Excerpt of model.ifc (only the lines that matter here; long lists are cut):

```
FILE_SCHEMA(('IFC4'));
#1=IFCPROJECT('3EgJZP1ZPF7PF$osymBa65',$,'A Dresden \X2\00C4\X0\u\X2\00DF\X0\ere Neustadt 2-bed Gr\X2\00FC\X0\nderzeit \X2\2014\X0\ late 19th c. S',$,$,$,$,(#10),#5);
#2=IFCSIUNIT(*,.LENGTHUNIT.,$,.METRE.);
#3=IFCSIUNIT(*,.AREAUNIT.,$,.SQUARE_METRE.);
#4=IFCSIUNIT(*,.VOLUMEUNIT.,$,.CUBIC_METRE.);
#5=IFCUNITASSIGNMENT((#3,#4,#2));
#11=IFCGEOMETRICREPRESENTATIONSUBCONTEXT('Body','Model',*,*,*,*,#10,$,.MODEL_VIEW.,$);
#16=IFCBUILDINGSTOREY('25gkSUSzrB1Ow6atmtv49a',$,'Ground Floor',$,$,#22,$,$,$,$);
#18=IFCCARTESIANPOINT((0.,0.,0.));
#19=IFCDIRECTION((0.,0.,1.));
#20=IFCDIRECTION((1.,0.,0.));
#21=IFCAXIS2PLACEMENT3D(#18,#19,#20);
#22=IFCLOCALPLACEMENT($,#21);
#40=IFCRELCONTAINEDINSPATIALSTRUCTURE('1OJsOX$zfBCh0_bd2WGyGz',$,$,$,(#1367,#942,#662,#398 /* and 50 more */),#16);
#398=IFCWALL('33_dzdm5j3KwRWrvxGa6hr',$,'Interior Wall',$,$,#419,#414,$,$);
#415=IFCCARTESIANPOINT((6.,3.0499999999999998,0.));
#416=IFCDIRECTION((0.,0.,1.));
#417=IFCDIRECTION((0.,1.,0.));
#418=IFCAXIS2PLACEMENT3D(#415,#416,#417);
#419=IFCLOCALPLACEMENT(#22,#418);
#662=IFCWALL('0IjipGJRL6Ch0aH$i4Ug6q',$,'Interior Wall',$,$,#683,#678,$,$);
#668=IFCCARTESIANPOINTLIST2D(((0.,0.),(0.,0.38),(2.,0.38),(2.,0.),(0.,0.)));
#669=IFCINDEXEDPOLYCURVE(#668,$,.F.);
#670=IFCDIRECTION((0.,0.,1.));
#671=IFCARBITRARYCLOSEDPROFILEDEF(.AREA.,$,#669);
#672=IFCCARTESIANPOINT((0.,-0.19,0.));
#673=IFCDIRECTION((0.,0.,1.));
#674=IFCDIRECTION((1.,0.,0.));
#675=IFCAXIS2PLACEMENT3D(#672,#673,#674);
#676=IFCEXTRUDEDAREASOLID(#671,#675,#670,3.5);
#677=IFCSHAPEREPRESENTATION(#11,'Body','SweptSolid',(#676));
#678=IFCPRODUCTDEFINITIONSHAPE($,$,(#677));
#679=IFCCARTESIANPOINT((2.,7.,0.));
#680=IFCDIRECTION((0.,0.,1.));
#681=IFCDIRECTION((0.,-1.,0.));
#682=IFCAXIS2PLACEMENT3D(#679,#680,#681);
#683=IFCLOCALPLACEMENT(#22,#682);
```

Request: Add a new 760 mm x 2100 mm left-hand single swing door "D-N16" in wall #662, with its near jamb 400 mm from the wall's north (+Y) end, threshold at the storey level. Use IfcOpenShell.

```python
import numpy as np
import ifcopenshell
import ifcopenshell.api.feature
import ifcopenshell.api.geometry
import ifcopenshell.api.root
import ifcopenshell.api.spatial
import ifcopenshell.geom
import ifcopenshell.util.element
import ifcopenshell.util.placement
import ifcopenshell.util.representation
import ifcopenshell.util.shape
import ifcopenshell.util.unit

model = ifcopenshell.open("model.ifc")
unit_scale = ifcopenshell.util.unit.calculate_unit_scale(model)
settings = ifcopenshell.geom.settings()


def volume(element):
    """Net volume in cubic metres, openings subtracted."""
    shape = ifcopenshell.geom.create_shape(settings, element)
    return ifcopenshell.util.shape.get_volume(shape.geometry)


wall = model.by_guid("0IjipGJRL6Ch0aH$i4Ug6q")
storey = ifcopenshell.util.element.get_container(wall, ifc_class="IfcBuildingStorey")
context = ifcopenshell.util.representation.get_context(model, "Model", "Body", "MODEL_VIEW")
before = volume(wall)

width, height, from_end, sill = 0.76, 2.1, 0.4, 0.0  # metres

# The wall runs along its own X axis, and the end named is its -X end.
wall_shape = ifcopenshell.geom.create_shape(settings, wall)
x, y, z = ifcopenshell.util.shape.get_vertices(wall_shape.geometry).T
start = x.min() + from_end
face, thickness = float(y.min()), float(y.max() - y.min())
wall_matrix = ifcopenshell.util.placement.get_local_placement(wall.ObjectPlacement)
level = ifcopenshell.util.placement.get_local_placement(storey.ObjectPlacement)[2, 3]


def in_wall(x, y):
    """Placement at x, y metres in the wall's axes, at sill height."""
    matrix = wall_matrix.copy()
    matrix[:, 3] = wall_matrix @ np.array([x / unit_scale, y / unit_scale, 0.0, 1.0])
    matrix[2, 3] = level + sill / unit_scale
    return matrix


# Opening: a box that overshoots both wall faces by 50 mm.
opening = ifcopenshell.api.root.create_entity(model, ifc_class="IfcOpeningElement", predefined_type="OPENING")
box = ifcopenshell.api.geometry.add_wall_representation(
    model, context=context, length=width, height=height, thickness=thickness + 0.1
)
ifcopenshell.api.geometry.assign_representation(model, product=opening, representation=box)
ifcopenshell.api.geometry.edit_object_placement(model, product=opening, matrix=in_wall(start, face - 0.05), is_si=False)
ifcopenshell.api.feature.add_feature(model, feature=opening, element=wall)

door = ifcopenshell.api.root.create_entity(model, ifc_class="IfcDoor", name="D-N16", predefined_type="DOOR")
door.OverallWidth, door.OverallHeight = width / unit_scale, height / unit_scale
door.OperationType = "SINGLE_SWING_LEFT"
body = ifcopenshell.api.geometry.add_door_representation(
    model,
    context=context,
    overall_width=door.OverallWidth,
    overall_height=door.OverallHeight,
    operation_type="SINGLE_SWING_LEFT",
    lining_properties={"LiningDepth": thickness / unit_scale, "ThresholdDepth": thickness / unit_scale},
)
ifcopenshell.api.geometry.assign_representation(model, product=door, representation=body)
ifcopenshell.api.spatial.assign_container(model, products=[door], relating_structure=storey)
ifcopenshell.api.feature.add_filling(model, opening=opening, element=door)

# The lining spans the wall, so the door starts at the wall face.
ifcopenshell.api.geometry.edit_object_placement(model, product=door, matrix=in_wall(start, face), is_si=False)

after = volume(wall)

print(f"wall volume {before:.3f} -> {after:.3f} m3")

model.write("model_updated.ifc")
```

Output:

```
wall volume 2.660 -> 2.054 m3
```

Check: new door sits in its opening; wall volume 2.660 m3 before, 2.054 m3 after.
